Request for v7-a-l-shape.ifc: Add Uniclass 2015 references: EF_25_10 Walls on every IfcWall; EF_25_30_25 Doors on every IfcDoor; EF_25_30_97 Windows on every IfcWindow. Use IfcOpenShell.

First a look at what the model holds.

```python
import ifcopenshell

model = ifcopenshell.open("v7-a-l-shape.ifc")
print(model.schema)
print("classifications:", [c.Name for c in model.by_type("IfcClassification")])
for ifc_class in ("IfcDoor", "IfcRoof", "IfcStair", "IfcWall", "IfcWindow"):
    print(ifc_class, len(model.by_type(ifc_class)))
```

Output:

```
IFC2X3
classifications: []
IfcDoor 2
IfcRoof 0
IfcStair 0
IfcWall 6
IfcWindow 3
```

```python
import ifcopenshell
import ifcopenshell.api.classification

model = ifcopenshell.open("v7-a-l-shape.ifc")

# IFC2X3 requires Source and Edition and has no link from the project to the system.
system = model.create_entity("IfcClassification", Source="NBS", Edition="2015", Name="Uniclass 2015")

codes = {
    "IfcWall": ("EF_25_10", "Walls"),
    "IfcDoor": ("EF_25_30_25", "Doors"),
    "IfcWindow": ("EF_25_30_97", "Windows"),
}
for ifc_class, (code, name) in codes.items():
    products = model.by_type(ifc_class)
    ifcopenshell.api.classification.add_reference(
        model, products=products, classification=system, identification=code, name=name
    )
    print(code, len(products))

model.write("v7-a-l-shape_updated.ifc")
```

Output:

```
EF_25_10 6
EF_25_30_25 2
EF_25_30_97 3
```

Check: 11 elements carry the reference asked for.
